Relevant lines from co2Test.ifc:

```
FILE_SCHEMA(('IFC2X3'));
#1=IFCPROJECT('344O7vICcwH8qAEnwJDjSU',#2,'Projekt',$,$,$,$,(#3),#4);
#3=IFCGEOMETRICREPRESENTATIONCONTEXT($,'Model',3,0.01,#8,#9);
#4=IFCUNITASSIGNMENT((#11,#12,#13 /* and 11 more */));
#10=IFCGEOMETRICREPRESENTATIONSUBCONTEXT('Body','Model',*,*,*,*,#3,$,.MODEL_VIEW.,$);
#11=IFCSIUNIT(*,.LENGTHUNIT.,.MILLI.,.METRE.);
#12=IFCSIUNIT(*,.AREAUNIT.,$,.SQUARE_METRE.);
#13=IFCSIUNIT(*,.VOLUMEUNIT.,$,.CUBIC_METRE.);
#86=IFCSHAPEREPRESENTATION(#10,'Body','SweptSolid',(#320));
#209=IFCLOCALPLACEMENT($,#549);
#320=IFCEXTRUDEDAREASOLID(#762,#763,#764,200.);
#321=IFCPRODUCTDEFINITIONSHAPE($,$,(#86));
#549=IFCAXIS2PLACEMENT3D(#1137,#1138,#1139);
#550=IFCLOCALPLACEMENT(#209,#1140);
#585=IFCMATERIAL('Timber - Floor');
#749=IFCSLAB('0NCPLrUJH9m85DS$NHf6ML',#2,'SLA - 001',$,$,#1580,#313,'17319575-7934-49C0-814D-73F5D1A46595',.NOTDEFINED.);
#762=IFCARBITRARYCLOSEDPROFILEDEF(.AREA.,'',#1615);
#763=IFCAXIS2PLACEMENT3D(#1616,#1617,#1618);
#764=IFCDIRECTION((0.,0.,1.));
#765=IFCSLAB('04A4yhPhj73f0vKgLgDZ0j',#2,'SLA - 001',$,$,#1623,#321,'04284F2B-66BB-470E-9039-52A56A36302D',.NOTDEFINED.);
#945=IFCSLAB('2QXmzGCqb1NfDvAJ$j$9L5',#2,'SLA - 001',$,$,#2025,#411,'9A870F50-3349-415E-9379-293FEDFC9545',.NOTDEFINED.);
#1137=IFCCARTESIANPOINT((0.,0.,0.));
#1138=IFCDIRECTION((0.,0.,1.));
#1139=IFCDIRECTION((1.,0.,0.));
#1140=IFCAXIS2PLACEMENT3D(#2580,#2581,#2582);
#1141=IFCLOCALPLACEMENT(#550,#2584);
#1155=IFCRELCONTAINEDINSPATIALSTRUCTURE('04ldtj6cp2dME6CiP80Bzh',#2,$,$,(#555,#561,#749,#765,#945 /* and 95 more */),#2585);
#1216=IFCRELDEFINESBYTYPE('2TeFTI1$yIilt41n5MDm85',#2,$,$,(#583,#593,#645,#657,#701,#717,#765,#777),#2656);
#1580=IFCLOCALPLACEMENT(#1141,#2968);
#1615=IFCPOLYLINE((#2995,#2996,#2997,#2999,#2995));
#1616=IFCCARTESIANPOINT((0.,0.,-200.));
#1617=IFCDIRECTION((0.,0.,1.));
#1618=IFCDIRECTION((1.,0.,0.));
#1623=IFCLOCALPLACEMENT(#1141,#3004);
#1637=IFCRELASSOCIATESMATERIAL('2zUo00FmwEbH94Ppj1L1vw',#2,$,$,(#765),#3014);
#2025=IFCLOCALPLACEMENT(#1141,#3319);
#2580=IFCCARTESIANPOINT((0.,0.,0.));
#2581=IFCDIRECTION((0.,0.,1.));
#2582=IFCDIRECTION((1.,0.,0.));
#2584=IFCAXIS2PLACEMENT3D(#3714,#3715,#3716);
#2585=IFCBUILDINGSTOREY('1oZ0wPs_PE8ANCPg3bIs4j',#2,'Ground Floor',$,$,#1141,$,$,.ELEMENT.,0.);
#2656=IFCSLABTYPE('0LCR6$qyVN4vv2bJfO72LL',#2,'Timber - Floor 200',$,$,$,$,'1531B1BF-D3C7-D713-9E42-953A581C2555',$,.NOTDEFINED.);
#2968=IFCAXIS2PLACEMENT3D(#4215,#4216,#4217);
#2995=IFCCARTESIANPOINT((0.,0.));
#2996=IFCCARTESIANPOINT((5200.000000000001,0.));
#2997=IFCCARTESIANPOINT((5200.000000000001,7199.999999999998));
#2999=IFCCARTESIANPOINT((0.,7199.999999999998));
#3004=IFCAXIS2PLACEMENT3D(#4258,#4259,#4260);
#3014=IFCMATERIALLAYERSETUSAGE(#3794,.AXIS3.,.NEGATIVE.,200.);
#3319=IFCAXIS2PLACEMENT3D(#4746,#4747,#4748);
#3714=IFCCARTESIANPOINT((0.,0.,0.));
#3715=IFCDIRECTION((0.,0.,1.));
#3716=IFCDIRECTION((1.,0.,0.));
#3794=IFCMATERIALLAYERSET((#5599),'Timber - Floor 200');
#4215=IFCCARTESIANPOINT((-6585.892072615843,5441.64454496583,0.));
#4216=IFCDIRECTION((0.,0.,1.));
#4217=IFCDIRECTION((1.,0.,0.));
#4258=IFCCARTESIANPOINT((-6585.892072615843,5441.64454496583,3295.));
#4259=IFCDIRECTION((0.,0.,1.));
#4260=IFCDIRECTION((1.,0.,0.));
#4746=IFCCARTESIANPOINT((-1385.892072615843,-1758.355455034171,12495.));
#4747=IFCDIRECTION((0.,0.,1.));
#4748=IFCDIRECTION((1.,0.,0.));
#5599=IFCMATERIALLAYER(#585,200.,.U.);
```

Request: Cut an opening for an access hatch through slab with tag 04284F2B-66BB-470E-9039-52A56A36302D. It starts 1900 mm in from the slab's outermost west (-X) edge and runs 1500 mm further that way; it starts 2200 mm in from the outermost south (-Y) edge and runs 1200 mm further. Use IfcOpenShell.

```python
import numpy as np
import ifcopenshell
import ifcopenshell.api.feature
import ifcopenshell.api.geometry
import ifcopenshell.api.root
import ifcopenshell.geom
import ifcopenshell.util.placement
import ifcopenshell.util.representation
import ifcopenshell.util.shape
import ifcopenshell.util.unit

model = ifcopenshell.open("co2Test.ifc")
unit_scale = ifcopenshell.util.unit.calculate_unit_scale(model)
settings = ifcopenshell.geom.settings()


def volume(element):
    """Net volume in cubic metres, openings subtracted."""
    shape = ifcopenshell.geom.create_shape(settings, element)
    return ifcopenshell.util.shape.get_volume(shape.geometry)


slab = model.by_guid("04A4yhPhj73f0vKgLgDZ0j")
before = volume(slab)

# Extent in the slab's own axes, in metres. The edges named are its -X and -Y sides.
slab_shape = ifcopenshell.geom.create_shape(settings, slab)
vertices = ifcopenshell.util.shape.get_vertices(slab_shape.geometry)
x_min, y_min, bottom = vertices.min(axis=0)
top = vertices[:, 2].max()

opening = ifcopenshell.api.root.create_entity(model, ifc_class="IfcOpeningElement", name="Access hatch opening")
context = ifcopenshell.util.representation.get_context(model, "Model", "Body", "MODEL_VIEW")
width, depth = 1.5, 1.2
outline = [(0.0, 0.0), (width, 0.0), (width, depth), (0.0, depth), (0.0, 0.0)]
# Overshoot both faces by 50 mm so the cut is clean.
shape = ifcopenshell.api.geometry.add_slab_representation(
    model, context=context, depth=top - bottom + 0.1, polyline=outline
)
ifcopenshell.api.geometry.assign_representation(model, product=opening, representation=shape)

matrix = ifcopenshell.util.placement.get_local_placement(slab.ObjectPlacement)
matrix[:, 3] = matrix @ np.append(np.array([x_min + 1.9, y_min + 2.2, bottom - 0.05]) / unit_scale, 1.0)
ifcopenshell.api.geometry.edit_object_placement(model, product=opening, matrix=matrix, is_si=False)
ifcopenshell.api.feature.add_feature(model, feature=opening, element=slab)

after = volume(slab)

print(f"slab volume {before:.3f} -> {after:.3f} m3")

model.write("co2Test_rev.ifc")
```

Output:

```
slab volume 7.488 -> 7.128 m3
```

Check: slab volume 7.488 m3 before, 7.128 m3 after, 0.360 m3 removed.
